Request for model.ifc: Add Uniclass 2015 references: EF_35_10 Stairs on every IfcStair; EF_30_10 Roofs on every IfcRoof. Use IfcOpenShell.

First a look at what the model holds.

```python
import ifcopenshell

model = ifcopenshell.open("model.ifc")
print(model.schema)
print("classifications:", [c.Name for c in model.by_type("IfcClassification")])
for ifc_class in ("IfcDoor", "IfcRoof", "IfcStair", "IfcWall", "IfcWindow"):
    print(ifc_class, len(model.by_type(ifc_class)))
```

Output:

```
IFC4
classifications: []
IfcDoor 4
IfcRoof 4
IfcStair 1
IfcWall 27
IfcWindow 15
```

```python
import ifcopenshell
import ifcopenshell.api.classification

model = ifcopenshell.open("model.ifc")

system = ifcopenshell.api.classification.add_classification(model, classification="Uniclass 2015")

codes = {
    "IfcStair": ("EF_35_10", "Stairs"),
    "IfcRoof": ("EF_30_10", "Roofs"),
}
for ifc_class, (code, name) in codes.items():
    products = model.by_type(ifc_class)
    ifcopenshell.api.classification.add_reference(
        model, products=products, classification=system, identification=code, name=name
    )
    print(code, len(products))

model.write("model-out.ifc")
```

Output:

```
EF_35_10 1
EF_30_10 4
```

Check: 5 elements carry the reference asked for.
